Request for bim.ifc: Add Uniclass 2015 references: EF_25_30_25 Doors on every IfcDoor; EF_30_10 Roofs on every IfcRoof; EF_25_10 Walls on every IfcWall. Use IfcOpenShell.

First a look at what the model holds.

```python
import ifcopenshell

model = ifcopenshell.open("bim.ifc")
print(model.schema)
print("classifications:", [c.Name for c in model.by_type("IfcClassification")])
for ifc_class in ("IfcDoor", "IfcRoof", "IfcStair", "IfcWall", "IfcWindow"):
    print(ifc_class, len(model.by_type(ifc_class)))
```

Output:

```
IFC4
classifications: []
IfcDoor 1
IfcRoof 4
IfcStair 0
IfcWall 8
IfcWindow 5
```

```python
import ifcopenshell
import ifcopenshell.api.classification

model = ifcopenshell.open("bim.ifc")

system = ifcopenshell.api.classification.add_classification(model, classification="Uniclass 2015")

codes = {
    "IfcDoor": ("EF_25_30_25", "Doors"),
    "IfcRoof": ("EF_30_10", "Roofs"),
    "IfcWall": ("EF_25_10", "Walls"),
}
for ifc_class, (code, name) in codes.items():
    products = model.by_type(ifc_class)
    ifcopenshell.api.classification.add_reference(
        model, products=products, classification=system, identification=code, name=name
    )
    print(code, len(products))

model.write("bim-out.ifc")
```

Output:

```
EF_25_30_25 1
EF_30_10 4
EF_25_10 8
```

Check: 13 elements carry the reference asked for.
